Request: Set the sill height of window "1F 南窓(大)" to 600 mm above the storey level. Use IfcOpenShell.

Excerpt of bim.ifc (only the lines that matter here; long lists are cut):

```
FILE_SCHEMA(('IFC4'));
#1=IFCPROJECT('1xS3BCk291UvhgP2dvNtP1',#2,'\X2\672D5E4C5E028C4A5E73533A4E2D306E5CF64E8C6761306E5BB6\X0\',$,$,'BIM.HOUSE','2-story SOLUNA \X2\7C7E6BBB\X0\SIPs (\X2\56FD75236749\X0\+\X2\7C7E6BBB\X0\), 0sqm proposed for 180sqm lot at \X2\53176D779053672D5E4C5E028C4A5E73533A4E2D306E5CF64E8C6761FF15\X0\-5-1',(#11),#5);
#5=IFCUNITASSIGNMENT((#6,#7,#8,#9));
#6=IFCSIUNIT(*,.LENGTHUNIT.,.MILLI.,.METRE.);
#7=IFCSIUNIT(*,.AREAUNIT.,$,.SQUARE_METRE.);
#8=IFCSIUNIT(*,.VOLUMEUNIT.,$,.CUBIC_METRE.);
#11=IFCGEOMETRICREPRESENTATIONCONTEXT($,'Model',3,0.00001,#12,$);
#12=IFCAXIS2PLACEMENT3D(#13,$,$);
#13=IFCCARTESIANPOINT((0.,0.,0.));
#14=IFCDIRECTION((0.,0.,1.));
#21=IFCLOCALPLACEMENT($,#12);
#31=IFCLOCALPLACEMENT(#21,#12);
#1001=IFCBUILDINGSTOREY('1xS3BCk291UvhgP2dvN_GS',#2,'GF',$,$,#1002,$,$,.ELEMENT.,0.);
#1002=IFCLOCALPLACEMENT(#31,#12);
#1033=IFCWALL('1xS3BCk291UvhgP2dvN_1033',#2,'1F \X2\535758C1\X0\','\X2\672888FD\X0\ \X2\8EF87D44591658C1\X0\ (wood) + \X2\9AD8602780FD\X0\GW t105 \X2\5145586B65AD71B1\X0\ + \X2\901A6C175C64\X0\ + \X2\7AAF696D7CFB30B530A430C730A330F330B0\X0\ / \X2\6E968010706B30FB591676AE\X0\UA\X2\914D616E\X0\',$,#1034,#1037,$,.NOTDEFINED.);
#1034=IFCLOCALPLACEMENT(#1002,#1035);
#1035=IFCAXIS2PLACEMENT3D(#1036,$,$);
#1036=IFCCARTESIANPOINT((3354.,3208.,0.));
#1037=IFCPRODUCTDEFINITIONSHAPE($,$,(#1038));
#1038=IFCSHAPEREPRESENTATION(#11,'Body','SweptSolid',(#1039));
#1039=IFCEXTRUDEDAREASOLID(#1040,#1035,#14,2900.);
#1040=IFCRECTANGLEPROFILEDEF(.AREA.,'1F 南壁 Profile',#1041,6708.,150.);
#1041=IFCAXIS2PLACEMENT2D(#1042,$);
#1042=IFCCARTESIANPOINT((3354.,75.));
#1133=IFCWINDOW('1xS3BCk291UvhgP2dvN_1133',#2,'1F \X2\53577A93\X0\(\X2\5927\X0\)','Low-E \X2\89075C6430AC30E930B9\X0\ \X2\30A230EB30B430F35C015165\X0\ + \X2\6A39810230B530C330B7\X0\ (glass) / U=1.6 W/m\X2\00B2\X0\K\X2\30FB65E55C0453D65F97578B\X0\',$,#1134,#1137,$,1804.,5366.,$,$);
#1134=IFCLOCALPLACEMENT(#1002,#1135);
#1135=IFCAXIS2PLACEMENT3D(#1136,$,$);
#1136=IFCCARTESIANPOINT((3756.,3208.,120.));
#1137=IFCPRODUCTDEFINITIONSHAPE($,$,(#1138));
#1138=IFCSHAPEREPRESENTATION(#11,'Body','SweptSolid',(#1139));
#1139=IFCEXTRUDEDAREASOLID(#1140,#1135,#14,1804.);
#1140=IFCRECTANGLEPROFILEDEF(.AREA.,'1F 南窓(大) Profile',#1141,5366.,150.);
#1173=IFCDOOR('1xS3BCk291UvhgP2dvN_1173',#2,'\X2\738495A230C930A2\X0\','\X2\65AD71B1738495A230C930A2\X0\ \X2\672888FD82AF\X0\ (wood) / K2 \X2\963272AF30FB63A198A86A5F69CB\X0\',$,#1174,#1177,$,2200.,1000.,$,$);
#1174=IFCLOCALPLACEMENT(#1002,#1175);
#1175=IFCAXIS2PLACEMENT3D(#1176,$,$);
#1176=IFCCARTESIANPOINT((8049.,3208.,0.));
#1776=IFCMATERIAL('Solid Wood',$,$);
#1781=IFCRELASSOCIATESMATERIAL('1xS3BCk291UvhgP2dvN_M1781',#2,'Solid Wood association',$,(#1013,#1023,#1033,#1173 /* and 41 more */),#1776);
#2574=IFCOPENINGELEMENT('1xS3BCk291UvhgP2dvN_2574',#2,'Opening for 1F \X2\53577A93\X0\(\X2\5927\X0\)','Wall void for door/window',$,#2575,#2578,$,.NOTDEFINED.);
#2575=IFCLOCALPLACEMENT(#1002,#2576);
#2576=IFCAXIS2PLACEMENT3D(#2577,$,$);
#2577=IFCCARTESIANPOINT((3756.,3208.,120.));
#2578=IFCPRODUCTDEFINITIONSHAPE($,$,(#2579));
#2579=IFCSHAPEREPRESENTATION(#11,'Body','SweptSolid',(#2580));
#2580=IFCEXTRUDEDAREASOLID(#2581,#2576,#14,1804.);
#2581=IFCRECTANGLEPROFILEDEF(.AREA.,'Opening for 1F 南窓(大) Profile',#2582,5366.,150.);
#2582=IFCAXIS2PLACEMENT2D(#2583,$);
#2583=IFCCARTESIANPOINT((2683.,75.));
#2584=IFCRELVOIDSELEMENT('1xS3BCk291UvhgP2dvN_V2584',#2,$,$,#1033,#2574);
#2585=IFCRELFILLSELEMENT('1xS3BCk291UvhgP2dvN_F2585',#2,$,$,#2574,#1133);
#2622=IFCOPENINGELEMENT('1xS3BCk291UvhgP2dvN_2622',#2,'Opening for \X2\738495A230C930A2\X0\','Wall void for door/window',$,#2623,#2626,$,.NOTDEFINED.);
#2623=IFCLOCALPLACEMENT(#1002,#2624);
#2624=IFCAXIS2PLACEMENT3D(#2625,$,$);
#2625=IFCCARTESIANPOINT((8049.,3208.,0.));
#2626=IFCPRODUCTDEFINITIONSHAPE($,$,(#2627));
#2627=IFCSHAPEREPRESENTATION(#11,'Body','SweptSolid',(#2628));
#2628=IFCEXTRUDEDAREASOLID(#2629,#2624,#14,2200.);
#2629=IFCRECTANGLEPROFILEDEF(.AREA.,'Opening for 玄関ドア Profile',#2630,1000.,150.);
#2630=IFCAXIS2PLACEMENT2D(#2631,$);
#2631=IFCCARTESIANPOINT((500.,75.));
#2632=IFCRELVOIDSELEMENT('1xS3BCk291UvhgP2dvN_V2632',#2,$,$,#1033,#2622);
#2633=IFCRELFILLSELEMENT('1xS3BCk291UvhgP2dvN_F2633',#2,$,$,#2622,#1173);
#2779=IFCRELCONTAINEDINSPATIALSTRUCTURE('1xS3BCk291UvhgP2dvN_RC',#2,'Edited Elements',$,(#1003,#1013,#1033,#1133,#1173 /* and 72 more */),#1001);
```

```python
import numpy as np
import ifcopenshell
import ifcopenshell.api.geometry
import ifcopenshell.geom
import ifcopenshell.util.element
import ifcopenshell.util.placement
import ifcopenshell.util.shape
import ifcopenshell.util.unit

model = ifcopenshell.open("bim.ifc")
unit_scale = ifcopenshell.util.unit.calculate_unit_scale(model)

window = model.by_guid("1xS3BCk291UvhgP2dvN_1133")
opening = window.FillsVoids[0].RelatingOpeningElement
storey = ifcopenshell.util.element.get_container(window, ifc_class="IfcBuildingStorey")
level = ifcopenshell.util.placement.get_local_placement(storey.ObjectPlacement)[2, 3]

# The opening's origin need not be at the sill, so measure its lowest point.
shape = ifcopenshell.geom.create_shape(ifcopenshell.geom.settings(), opening)
bottom = ifcopenshell.util.shape.get_shape_bottom_elevation(shape, shape.geometry) / unit_scale
dz = level + 600.0 - bottom

shift = np.array([0.0, 0.0, dz])
# The window is not placed relative to its opening, so move both.
for product in (opening, window):
    matrix = ifcopenshell.util.placement.get_local_placement(product.ObjectPlacement)
    matrix[:3, 3] += shift
    ifcopenshell.api.geometry.edit_object_placement(model, product=product, matrix=matrix, is_si=False)

print(f"moved by {dz * unit_scale:+.3f} m")

model.write("bim_v2.ifc")
```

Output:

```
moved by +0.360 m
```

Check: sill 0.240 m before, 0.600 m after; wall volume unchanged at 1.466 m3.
